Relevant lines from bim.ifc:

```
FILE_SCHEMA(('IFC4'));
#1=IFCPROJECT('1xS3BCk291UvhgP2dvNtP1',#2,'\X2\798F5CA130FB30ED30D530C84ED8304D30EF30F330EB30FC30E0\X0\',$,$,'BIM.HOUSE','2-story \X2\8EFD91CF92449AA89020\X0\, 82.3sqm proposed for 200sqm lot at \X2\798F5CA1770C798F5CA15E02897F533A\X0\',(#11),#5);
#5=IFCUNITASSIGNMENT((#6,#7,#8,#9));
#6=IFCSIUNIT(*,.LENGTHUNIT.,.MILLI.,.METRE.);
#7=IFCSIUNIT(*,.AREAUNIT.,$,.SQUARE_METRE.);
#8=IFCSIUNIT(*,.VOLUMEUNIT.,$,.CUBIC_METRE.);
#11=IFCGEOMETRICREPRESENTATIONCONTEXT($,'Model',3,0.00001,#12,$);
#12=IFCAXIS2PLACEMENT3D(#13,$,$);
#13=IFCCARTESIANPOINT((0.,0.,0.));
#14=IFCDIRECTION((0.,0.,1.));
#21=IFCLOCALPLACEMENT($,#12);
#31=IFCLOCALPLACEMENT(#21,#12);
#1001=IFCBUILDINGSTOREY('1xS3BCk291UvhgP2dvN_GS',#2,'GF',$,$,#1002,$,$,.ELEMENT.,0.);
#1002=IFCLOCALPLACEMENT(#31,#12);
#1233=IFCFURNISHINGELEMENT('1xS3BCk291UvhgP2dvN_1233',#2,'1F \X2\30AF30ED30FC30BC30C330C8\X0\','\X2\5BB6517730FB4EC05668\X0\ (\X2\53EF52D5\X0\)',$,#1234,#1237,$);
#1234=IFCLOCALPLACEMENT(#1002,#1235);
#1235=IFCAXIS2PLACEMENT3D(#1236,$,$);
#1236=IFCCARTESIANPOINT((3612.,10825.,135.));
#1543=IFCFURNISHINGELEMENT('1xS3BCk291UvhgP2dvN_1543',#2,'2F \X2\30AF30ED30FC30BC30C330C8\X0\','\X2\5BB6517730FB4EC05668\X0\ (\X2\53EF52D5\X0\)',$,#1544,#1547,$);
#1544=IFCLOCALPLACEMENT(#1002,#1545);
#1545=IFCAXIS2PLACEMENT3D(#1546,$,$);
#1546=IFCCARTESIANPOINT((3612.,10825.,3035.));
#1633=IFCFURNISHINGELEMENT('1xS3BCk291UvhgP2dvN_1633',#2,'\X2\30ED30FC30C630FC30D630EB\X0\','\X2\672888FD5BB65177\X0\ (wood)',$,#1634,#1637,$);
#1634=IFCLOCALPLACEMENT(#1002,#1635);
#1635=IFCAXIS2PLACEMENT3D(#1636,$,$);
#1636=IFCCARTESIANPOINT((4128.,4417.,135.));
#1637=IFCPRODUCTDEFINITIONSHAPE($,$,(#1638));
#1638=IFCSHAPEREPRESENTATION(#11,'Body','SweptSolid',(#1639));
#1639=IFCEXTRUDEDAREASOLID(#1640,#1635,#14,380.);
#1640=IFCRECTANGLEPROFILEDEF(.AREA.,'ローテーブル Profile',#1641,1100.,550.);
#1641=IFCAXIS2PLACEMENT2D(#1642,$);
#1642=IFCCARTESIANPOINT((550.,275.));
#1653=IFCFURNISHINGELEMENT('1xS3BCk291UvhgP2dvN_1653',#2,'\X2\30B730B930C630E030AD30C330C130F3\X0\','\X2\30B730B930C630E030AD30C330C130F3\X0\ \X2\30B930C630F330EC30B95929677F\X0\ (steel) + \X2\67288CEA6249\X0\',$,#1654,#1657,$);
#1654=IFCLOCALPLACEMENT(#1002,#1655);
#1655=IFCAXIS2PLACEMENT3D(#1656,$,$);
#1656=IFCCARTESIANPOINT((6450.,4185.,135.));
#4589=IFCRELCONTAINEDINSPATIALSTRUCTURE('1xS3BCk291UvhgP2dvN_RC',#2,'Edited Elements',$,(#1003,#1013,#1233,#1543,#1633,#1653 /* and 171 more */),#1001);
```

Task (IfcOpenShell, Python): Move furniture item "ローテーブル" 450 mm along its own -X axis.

```python
import ifcopenshell
import ifcopenshell.api.geometry
import ifcopenshell.util.placement

model = ifcopenshell.open("bim.ifc")

item = model.by_guid("1xS3BCk291UvhgP2dvN_1633")
matrix = ifcopenshell.util.placement.get_local_placement(item.ObjectPlacement)
matrix[:3, 3] -= matrix[:3, 0] * 450.0
ifcopenshell.api.geometry.edit_object_placement(model, product=item, matrix=matrix, is_si=False)

print(ifcopenshell.util.placement.get_local_placement(item.ObjectPlacement).round(3) + 0.0)

model.write("bim_v2.ifc")
```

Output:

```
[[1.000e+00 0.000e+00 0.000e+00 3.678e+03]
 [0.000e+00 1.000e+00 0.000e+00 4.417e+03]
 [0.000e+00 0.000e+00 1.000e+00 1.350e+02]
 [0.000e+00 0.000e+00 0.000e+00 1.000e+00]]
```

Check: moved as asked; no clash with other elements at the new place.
